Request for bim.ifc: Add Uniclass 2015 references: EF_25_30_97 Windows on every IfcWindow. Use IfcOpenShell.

First a look at what the model holds.

```python
import ifcopenshell

model = ifcopenshell.open("bim.ifc")
print(model.schema)
print("classifications:", [c.Name for c in model.by_type("IfcClassification")])
for ifc_class in ("IfcDoor", "IfcRoof", "IfcStair", "IfcWall", "IfcWindow"):
    print(ifc_class, len(model.by_type(ifc_class)))
```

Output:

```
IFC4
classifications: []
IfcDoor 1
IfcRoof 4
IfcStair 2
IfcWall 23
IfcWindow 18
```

```python
import ifcopenshell
import ifcopenshell.api.classification

model = ifcopenshell.open("bim.ifc")

system = ifcopenshell.api.classification.add_classification(model, classification="Uniclass 2015")

codes = {
    "IfcWindow": ("EF_25_30_97", "Windows"),
}
for ifc_class, (code, name) in codes.items():
    products = model.by_type(ifc_class)
    ifcopenshell.api.classification.add_reference(
        model, products=products, classification=system, identification=code, name=name
    )
    print(code, len(products))

model.write("bim_updated.ifc")
```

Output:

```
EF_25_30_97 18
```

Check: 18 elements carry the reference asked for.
